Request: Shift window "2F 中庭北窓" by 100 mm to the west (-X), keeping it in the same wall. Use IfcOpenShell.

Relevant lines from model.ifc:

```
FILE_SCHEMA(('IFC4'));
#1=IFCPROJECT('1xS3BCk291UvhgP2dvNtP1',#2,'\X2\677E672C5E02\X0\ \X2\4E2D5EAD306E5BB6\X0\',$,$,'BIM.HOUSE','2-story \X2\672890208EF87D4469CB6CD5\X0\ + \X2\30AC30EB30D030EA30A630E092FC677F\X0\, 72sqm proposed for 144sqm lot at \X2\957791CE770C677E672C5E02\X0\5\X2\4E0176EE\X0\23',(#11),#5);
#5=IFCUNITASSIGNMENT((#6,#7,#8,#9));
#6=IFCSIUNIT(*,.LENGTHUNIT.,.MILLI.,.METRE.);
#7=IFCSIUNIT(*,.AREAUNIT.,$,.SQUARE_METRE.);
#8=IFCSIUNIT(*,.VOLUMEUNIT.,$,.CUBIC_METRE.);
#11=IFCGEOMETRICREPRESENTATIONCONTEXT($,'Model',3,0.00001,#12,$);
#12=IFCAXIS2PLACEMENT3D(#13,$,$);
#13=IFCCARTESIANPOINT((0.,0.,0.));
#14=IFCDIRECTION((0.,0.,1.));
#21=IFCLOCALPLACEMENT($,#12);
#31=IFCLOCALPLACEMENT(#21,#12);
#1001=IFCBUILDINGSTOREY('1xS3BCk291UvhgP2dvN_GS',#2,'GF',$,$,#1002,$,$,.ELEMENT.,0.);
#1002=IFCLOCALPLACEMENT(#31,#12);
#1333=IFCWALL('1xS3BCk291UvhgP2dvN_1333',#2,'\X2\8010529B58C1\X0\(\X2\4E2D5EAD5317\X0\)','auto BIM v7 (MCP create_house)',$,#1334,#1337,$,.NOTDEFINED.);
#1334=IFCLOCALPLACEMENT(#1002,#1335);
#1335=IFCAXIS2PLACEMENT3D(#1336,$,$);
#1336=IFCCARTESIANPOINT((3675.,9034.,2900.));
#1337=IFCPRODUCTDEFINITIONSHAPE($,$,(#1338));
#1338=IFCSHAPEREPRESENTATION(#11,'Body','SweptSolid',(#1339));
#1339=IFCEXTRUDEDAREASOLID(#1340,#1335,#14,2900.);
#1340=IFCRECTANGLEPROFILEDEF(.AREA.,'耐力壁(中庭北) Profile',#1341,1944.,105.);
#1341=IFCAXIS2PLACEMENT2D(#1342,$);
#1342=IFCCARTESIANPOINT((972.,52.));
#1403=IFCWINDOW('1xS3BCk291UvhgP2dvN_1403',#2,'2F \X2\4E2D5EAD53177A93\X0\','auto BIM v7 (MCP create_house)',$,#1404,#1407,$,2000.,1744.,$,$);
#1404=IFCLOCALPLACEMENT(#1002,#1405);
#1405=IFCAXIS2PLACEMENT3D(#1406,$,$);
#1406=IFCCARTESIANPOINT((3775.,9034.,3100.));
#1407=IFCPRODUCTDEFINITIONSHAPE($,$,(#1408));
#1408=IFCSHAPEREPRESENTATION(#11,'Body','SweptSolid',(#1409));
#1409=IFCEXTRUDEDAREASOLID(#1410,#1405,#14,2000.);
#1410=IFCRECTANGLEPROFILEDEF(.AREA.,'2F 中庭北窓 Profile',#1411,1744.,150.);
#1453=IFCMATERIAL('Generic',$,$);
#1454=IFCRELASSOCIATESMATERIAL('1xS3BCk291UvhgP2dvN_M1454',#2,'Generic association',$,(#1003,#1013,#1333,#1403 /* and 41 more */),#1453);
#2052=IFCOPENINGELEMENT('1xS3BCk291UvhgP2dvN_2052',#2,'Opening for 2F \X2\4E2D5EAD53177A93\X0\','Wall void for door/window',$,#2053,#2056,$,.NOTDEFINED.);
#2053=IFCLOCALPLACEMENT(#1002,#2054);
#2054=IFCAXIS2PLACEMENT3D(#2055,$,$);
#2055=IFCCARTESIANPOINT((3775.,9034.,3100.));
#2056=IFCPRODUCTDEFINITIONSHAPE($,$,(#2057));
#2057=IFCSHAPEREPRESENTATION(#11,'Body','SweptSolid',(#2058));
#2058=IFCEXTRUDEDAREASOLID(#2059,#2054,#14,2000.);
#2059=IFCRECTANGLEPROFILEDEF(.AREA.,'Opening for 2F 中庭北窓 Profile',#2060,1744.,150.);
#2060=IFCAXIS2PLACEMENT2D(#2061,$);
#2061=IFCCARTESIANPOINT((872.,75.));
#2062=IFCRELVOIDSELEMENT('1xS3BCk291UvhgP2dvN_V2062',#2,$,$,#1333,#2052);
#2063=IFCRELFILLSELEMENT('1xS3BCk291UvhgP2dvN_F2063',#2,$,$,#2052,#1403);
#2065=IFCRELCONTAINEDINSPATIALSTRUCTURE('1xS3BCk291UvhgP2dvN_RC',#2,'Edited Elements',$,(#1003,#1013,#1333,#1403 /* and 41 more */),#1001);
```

```python
import ifcopenshell
import ifcopenshell.api.geometry
import ifcopenshell.util.placement

model = ifcopenshell.open("model.ifc")

window = model.by_guid("1xS3BCk291UvhgP2dvN_1403")
opening = window.FillsVoids[0].RelatingOpeningElement
wall = opening.VoidsElements[0].RelatingBuildingElement

wall_matrix = ifcopenshell.util.placement.get_local_placement(wall.ObjectPlacement)
shift = wall_matrix[:3, 0] * -100.0
before = ifcopenshell.util.placement.get_local_placement(window.ObjectPlacement)[:3, 3].copy()

# The window is not placed relative to its opening, so move both.
for product in (opening, window):
    matrix = ifcopenshell.util.placement.get_local_placement(product.ObjectPlacement)
    matrix[:3, 3] += shift
    ifcopenshell.api.geometry.edit_object_placement(model, product=product, matrix=matrix, is_si=False)

after = ifcopenshell.util.placement.get_local_placement(window.ObjectPlacement)[:3, 3]
print("window moved by", (after - before).round(3) + 0.0)

model.write("model-out.ifc")
```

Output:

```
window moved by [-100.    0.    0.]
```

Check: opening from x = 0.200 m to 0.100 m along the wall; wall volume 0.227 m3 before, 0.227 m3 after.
